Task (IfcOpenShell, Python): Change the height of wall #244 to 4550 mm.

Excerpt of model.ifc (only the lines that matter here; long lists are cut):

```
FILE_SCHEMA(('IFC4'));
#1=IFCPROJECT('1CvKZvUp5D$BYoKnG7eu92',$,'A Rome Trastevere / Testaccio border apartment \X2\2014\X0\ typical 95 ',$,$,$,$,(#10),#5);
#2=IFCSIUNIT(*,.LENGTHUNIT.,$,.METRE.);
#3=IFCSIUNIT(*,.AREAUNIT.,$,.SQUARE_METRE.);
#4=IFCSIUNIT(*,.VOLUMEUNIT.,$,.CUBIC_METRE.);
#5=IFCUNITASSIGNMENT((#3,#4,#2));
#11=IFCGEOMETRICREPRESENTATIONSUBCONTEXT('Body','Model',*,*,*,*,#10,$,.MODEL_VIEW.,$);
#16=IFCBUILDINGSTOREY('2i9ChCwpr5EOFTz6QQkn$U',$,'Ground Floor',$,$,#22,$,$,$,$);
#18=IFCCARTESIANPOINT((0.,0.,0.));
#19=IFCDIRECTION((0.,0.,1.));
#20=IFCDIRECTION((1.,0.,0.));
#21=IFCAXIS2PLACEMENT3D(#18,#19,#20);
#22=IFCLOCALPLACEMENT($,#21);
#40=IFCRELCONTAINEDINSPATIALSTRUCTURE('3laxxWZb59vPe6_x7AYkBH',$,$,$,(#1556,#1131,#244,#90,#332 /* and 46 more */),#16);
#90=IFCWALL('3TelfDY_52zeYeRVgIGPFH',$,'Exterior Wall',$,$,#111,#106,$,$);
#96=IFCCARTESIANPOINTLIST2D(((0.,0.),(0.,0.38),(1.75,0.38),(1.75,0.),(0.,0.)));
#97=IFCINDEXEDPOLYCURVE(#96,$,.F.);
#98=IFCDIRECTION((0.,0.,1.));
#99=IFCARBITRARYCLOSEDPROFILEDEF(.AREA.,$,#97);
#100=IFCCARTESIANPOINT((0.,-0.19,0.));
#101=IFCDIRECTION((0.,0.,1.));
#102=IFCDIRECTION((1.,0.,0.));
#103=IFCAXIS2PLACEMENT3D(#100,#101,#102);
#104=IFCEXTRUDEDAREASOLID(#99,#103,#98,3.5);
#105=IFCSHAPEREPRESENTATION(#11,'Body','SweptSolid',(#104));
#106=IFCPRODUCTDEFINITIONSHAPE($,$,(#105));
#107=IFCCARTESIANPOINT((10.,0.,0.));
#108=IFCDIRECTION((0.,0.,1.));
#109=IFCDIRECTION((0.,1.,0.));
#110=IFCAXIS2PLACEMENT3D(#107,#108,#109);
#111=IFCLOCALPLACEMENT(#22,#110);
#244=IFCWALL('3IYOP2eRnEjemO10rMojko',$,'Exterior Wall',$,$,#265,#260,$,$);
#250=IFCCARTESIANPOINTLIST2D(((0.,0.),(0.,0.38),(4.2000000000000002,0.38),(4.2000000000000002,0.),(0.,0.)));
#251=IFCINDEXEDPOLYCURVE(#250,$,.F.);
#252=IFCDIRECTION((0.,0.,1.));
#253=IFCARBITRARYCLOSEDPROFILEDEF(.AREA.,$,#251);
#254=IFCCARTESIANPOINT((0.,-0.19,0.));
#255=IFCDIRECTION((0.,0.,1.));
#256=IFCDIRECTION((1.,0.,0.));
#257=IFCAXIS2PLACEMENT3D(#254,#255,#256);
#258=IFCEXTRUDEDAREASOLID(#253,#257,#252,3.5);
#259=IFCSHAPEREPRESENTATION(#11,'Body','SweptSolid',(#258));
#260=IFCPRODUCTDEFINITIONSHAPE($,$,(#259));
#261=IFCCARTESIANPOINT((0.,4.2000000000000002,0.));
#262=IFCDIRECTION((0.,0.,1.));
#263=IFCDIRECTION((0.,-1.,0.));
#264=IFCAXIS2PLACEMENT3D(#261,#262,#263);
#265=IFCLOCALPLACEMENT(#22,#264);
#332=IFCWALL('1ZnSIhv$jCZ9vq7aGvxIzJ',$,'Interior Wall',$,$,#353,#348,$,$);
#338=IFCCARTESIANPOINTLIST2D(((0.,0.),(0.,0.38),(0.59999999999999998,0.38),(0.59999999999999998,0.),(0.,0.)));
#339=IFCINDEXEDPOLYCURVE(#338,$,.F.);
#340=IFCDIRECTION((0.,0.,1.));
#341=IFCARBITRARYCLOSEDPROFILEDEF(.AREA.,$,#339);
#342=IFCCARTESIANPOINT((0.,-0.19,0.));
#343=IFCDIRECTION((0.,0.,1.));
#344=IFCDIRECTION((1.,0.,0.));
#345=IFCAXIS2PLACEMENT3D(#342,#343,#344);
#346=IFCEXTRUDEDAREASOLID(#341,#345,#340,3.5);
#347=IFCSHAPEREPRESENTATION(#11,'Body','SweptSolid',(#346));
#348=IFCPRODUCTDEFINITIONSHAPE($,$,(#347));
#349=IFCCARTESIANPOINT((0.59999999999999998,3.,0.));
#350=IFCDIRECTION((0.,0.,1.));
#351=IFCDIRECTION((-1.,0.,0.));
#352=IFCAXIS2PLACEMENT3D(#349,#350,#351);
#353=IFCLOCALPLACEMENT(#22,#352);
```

```python
import ifcopenshell
import ifcopenshell.geom
import ifcopenshell.util.representation
import ifcopenshell.util.shape
import ifcopenshell.util.unit

model = ifcopenshell.open("model.ifc")
unit_scale = ifcopenshell.util.unit.calculate_unit_scale(model)
settings = ifcopenshell.geom.settings()


def volume(element):
    """Net volume in cubic metres, openings subtracted."""
    shape = ifcopenshell.geom.create_shape(settings, element)
    return ifcopenshell.util.shape.get_volume(shape.geometry)


wall = model.by_id(244)
before = volume(wall)

body = ifcopenshell.util.representation.get_representation(wall, "Model", "Body")
solid = body.Items[0]
old_height = solid.Depth
solid.Depth = 4.55 / unit_scale
after = volume(wall)

print(f"height {old_height:g} -> {solid.Depth:g}, volume {before:.3f} -> {after:.3f} m3")

model.write("model_edited.ifc")
```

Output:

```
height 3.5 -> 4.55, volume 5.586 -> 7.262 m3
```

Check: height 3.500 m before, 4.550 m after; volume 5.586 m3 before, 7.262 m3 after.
